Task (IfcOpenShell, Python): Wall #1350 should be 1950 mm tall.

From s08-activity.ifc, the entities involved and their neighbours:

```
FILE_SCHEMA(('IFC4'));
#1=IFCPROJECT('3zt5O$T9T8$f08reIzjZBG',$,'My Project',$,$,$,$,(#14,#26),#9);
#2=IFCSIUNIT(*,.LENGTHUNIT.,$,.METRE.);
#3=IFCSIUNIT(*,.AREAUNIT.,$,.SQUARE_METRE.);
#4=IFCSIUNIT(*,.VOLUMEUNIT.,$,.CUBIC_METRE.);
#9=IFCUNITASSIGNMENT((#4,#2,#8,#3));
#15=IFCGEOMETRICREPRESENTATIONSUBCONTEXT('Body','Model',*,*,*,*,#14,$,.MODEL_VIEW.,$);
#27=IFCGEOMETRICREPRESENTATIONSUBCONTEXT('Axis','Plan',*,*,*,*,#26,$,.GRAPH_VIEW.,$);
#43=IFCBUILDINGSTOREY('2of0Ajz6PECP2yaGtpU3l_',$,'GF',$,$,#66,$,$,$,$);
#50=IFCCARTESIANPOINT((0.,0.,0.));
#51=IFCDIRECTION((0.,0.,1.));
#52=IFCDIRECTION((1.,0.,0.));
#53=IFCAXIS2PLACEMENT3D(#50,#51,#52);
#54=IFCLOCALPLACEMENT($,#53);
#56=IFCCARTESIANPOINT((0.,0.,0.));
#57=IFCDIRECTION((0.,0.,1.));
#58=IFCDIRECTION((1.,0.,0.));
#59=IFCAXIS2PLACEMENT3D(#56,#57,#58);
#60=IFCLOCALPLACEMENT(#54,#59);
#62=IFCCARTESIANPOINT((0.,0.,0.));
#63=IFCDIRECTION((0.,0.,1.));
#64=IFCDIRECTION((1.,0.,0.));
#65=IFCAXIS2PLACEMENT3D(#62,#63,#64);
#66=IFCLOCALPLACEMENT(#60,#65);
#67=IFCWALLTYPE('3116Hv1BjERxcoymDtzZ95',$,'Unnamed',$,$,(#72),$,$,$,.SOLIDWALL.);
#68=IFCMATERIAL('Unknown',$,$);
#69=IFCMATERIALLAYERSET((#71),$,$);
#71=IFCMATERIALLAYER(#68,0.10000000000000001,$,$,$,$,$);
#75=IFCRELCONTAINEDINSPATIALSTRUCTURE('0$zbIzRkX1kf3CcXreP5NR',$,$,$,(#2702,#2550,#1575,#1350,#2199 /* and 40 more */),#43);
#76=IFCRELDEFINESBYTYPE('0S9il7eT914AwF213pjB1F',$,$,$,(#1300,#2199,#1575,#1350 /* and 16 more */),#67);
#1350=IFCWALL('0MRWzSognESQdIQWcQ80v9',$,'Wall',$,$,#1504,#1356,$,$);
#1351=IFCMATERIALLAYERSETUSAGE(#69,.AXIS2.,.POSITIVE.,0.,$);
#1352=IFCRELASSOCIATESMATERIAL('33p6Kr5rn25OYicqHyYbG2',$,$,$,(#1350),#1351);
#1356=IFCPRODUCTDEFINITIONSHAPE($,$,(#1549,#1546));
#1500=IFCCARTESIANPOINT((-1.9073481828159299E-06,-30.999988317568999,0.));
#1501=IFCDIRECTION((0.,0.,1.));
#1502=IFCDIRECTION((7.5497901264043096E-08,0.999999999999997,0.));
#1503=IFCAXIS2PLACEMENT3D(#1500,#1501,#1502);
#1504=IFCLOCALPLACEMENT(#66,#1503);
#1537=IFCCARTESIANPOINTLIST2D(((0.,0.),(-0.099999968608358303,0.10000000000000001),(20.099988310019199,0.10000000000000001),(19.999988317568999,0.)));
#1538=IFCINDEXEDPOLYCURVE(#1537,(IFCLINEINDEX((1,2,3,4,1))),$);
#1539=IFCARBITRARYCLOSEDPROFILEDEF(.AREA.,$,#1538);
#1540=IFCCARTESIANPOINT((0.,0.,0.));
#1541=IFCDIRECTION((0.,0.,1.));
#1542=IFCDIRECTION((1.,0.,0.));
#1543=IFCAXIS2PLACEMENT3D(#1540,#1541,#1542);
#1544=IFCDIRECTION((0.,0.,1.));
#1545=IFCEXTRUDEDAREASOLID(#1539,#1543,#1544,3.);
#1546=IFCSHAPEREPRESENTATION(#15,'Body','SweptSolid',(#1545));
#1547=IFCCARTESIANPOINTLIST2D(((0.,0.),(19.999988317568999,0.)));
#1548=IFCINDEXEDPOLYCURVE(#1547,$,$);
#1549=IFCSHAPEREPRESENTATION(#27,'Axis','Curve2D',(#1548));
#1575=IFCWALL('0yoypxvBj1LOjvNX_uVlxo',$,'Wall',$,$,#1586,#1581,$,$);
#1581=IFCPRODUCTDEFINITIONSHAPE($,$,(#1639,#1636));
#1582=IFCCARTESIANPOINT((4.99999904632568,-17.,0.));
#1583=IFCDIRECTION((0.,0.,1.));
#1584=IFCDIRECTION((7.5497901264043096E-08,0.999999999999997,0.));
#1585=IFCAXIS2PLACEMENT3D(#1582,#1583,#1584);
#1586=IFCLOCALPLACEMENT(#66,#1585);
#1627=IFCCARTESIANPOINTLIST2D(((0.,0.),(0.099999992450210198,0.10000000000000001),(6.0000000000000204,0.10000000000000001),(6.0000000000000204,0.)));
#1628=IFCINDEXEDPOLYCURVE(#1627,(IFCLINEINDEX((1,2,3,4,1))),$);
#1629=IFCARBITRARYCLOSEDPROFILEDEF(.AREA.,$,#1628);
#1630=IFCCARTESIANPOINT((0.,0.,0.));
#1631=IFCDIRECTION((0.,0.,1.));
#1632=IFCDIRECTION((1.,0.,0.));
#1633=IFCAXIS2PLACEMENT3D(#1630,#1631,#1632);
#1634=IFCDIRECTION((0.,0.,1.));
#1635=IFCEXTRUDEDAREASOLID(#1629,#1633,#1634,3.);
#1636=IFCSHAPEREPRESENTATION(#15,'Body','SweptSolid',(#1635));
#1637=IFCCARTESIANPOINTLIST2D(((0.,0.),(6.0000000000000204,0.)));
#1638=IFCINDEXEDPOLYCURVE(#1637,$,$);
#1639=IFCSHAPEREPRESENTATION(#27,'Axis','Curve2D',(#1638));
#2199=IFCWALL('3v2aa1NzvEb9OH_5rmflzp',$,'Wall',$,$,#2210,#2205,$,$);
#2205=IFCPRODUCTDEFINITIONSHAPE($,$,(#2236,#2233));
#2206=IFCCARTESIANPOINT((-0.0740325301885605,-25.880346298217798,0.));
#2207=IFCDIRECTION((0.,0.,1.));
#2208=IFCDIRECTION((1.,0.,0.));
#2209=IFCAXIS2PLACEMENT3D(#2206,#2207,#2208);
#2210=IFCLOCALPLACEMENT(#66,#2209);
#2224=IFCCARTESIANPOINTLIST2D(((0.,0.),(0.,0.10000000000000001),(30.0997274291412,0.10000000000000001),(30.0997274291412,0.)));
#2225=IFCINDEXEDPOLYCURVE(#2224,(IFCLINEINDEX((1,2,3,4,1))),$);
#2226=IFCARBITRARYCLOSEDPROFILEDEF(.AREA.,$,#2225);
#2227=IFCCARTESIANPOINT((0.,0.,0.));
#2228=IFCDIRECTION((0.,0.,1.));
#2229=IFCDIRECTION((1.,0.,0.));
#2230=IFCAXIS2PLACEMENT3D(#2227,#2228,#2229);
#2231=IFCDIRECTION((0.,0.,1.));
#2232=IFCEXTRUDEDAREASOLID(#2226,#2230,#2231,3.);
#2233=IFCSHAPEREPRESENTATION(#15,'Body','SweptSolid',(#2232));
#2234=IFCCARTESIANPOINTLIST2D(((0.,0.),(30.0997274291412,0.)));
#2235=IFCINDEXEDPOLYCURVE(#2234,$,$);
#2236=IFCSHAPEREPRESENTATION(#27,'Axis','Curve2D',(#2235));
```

```python
import ifcopenshell
import ifcopenshell.geom
import ifcopenshell.util.representation
import ifcopenshell.util.shape

model = ifcopenshell.open("s08-activity.ifc")
settings = ifcopenshell.geom.settings()


def volume(element):
    """Net volume in cubic metres, openings subtracted."""
    shape = ifcopenshell.geom.create_shape(settings, element)
    return ifcopenshell.util.shape.get_volume(shape.geometry)


wall = model.by_guid("0MRWzSognESQdIQWcQ80v9")
before = volume(wall)

body = ifcopenshell.util.representation.get_representation(wall, "Model", "Body")
solid = body.Items[0]
old_height = solid.Depth
solid.Depth = 1.95
after = volume(wall)

print(f"height {old_height:g} -> {solid.Depth:g}, volume {before:.3f} -> {after:.3f} m3")

model.write("s08-activity-out.ifc")
```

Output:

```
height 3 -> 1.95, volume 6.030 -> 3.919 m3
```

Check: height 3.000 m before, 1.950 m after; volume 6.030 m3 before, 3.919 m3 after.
